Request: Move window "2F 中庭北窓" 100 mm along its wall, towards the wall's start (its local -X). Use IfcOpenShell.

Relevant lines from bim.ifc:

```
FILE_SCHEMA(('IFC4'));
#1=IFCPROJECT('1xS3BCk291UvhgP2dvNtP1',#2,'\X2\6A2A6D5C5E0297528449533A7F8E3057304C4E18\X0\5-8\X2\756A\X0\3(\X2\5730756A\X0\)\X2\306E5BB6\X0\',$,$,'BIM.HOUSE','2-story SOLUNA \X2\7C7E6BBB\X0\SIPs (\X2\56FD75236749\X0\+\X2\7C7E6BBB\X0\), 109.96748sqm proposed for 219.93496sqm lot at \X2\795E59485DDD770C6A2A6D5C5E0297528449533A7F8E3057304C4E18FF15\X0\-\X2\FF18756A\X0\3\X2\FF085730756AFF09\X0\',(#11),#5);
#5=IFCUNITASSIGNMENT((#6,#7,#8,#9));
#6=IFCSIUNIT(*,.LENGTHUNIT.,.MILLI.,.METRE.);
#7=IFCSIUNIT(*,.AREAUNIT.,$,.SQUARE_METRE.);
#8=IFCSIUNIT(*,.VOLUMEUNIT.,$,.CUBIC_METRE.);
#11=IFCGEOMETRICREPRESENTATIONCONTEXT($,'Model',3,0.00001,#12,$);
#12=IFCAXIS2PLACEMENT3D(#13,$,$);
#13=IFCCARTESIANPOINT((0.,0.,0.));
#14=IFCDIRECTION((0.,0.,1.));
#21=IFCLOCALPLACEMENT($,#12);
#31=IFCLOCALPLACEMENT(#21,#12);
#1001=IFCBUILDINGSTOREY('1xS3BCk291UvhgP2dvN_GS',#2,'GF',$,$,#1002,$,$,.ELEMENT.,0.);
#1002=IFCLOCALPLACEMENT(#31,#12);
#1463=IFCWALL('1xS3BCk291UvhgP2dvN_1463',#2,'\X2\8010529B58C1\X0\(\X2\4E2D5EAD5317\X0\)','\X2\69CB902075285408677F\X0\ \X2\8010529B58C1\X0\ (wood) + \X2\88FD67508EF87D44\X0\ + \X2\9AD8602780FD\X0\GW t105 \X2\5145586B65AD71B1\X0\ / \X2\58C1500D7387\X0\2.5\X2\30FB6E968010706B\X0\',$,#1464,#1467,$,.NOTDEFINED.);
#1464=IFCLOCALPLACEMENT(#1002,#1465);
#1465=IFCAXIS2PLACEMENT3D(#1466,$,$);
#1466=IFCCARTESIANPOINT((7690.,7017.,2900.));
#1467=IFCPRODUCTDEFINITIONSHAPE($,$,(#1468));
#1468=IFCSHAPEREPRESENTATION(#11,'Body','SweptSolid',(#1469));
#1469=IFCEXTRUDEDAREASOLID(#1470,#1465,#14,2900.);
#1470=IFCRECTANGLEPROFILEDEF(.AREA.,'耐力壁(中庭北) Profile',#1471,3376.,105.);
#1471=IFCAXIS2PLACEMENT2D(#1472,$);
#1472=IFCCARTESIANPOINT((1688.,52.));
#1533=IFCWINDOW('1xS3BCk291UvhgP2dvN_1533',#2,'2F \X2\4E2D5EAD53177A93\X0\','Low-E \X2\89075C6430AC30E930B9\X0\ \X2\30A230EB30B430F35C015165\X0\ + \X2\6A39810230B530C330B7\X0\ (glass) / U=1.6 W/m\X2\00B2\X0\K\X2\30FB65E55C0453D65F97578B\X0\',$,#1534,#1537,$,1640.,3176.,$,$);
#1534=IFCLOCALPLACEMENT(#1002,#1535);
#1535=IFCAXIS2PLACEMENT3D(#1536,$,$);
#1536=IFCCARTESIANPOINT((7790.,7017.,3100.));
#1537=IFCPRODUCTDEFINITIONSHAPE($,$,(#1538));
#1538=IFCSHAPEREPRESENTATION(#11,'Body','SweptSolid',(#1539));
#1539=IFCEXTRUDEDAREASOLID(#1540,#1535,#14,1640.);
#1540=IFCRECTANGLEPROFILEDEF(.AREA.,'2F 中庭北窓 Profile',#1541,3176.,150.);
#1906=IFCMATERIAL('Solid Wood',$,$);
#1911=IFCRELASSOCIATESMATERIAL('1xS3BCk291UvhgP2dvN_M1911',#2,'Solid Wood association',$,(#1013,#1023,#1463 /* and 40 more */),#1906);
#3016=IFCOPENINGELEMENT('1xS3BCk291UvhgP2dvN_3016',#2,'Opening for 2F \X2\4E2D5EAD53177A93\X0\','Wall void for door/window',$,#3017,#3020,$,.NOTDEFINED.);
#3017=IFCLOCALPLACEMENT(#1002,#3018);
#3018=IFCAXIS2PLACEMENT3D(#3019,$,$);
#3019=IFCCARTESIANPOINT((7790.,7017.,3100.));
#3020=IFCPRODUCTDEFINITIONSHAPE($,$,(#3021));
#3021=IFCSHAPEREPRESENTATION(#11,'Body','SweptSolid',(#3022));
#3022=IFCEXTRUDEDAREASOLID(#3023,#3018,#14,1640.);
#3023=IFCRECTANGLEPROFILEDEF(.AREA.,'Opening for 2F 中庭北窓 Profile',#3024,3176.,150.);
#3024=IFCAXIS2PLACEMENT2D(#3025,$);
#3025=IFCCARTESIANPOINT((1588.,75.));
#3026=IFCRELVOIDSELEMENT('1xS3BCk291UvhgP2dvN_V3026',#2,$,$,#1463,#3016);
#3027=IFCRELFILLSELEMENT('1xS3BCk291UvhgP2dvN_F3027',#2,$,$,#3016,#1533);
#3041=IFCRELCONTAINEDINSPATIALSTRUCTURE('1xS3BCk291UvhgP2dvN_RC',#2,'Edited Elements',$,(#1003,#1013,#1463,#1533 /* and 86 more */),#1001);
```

```python
import ifcopenshell
import ifcopenshell.api.geometry
import ifcopenshell.util.placement
import ifcopenshell.util.unit

model = ifcopenshell.open("bim.ifc")
unit_scale = ifcopenshell.util.unit.calculate_unit_scale(model)

window = model.by_guid("1xS3BCk291UvhgP2dvN_1533")
opening = window.FillsVoids[0].RelatingOpeningElement
wall = opening.VoidsElements[0].RelatingBuildingElement

wall_matrix = ifcopenshell.util.placement.get_local_placement(wall.ObjectPlacement)
shift = wall_matrix[:3, 0] * -0.1 / unit_scale
before = ifcopenshell.util.placement.get_local_placement(window.ObjectPlacement)[:3, 3].copy()

# The window is not placed relative to its opening, so move both.
for product in (opening, window):
    matrix = ifcopenshell.util.placement.get_local_placement(product.ObjectPlacement)
    matrix[:3, 3] += shift
    ifcopenshell.api.geometry.edit_object_placement(model, product=product, matrix=matrix, is_si=False)

after = ifcopenshell.util.placement.get_local_placement(window.ObjectPlacement)[:3, 3]
print("window moved by", (after - before).round(3) + 0.0)

model.write("bim-out.ifc")
```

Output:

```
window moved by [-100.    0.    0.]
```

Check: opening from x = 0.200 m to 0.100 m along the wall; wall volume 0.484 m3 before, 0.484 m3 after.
